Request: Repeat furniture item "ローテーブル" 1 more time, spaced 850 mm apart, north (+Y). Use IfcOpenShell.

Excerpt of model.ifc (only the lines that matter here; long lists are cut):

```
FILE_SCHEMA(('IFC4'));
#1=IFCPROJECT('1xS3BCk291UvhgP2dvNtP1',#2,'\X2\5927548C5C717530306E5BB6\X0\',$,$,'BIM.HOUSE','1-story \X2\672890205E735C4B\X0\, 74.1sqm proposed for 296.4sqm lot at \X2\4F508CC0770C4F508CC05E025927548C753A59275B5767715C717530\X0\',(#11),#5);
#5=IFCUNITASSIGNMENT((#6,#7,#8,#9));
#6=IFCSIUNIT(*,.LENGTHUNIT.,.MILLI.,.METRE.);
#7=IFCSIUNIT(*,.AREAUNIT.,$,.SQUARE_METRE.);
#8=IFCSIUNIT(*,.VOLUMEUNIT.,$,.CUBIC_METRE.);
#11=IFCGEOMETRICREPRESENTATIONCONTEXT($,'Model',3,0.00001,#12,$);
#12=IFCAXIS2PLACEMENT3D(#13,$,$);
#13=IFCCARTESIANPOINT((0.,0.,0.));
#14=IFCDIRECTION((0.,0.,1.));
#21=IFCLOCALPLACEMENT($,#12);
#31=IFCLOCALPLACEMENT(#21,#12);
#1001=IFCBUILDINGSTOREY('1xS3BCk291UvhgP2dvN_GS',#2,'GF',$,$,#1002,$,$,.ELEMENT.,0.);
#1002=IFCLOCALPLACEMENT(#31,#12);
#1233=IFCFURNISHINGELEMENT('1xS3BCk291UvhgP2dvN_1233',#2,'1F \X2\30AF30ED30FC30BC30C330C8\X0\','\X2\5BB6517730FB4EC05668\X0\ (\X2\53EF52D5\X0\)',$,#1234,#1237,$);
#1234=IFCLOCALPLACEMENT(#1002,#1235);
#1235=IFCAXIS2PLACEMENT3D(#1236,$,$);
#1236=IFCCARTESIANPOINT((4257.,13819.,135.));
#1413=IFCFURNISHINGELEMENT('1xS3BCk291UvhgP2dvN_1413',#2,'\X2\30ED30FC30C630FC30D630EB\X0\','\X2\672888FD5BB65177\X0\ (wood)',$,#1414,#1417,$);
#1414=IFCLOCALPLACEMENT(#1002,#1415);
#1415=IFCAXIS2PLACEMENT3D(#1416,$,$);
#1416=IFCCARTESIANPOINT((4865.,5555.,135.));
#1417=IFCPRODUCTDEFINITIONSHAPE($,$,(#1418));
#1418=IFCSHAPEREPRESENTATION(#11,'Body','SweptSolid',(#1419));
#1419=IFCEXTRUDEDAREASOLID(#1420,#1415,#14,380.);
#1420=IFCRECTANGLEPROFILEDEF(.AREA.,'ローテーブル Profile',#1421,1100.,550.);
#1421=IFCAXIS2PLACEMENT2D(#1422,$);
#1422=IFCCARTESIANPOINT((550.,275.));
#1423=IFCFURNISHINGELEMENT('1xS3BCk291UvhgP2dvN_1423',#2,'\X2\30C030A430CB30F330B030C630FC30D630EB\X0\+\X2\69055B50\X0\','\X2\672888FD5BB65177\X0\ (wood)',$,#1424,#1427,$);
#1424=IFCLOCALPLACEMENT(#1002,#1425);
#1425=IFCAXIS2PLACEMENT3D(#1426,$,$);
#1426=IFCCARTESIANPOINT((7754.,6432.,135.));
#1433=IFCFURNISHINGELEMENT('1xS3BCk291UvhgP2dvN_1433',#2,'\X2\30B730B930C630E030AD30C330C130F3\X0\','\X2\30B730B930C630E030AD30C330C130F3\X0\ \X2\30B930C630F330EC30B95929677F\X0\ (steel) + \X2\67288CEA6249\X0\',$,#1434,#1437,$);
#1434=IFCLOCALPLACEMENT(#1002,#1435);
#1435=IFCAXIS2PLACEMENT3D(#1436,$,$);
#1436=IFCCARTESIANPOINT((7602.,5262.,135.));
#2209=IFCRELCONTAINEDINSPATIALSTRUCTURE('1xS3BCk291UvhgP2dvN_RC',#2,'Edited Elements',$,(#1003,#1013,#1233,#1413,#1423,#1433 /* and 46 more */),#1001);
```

```python
import numpy as np
import ifcopenshell
import ifcopenshell.api.geometry
import ifcopenshell.api.root
import ifcopenshell.util.element
import ifcopenshell.util.placement

model = ifcopenshell.open("model.ifc")


def reuse_history(source, copy):
    """copy_class also copies each property set's owner history, people and application; keep the originals."""
    for rel in copy.IsDefinedBy:
        if rel.is_a("IfcRelDefinesByProperties") and (history := rel.RelatingPropertyDefinition.OwnerHistory):
            rel.RelatingPropertyDefinition.OwnerHistory = source.OwnerHistory
            ifcopenshell.util.element.remove_deep2(model, history)


source = model.by_guid("1xS3BCk291UvhgP2dvN_1413")
base = ifcopenshell.util.placement.get_local_placement(source.ObjectPlacement)
step = np.array([0.0, 1.0, 0.0]) * 850.0

for i in range(1, 2):
    copy = ifcopenshell.api.root.copy_class(model, product=source)
    copy.Representation = ifcopenshell.util.element.copy_deep(
        model, source.Representation, exclude=["IfcGeometricRepresentationContext", "IfcRepresentationMap"]
    )
    reuse_history(source, copy)
    matrix = base.copy()
    matrix[:3, 3] += i * step
    print("added at", matrix[:3, 3].round(3) + 0.0)
    ifcopenshell.api.geometry.edit_object_placement(model, product=copy, matrix=matrix, is_si=False)

model.write("model_edited.ifc")
```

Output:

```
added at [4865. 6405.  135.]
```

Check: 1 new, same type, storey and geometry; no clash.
